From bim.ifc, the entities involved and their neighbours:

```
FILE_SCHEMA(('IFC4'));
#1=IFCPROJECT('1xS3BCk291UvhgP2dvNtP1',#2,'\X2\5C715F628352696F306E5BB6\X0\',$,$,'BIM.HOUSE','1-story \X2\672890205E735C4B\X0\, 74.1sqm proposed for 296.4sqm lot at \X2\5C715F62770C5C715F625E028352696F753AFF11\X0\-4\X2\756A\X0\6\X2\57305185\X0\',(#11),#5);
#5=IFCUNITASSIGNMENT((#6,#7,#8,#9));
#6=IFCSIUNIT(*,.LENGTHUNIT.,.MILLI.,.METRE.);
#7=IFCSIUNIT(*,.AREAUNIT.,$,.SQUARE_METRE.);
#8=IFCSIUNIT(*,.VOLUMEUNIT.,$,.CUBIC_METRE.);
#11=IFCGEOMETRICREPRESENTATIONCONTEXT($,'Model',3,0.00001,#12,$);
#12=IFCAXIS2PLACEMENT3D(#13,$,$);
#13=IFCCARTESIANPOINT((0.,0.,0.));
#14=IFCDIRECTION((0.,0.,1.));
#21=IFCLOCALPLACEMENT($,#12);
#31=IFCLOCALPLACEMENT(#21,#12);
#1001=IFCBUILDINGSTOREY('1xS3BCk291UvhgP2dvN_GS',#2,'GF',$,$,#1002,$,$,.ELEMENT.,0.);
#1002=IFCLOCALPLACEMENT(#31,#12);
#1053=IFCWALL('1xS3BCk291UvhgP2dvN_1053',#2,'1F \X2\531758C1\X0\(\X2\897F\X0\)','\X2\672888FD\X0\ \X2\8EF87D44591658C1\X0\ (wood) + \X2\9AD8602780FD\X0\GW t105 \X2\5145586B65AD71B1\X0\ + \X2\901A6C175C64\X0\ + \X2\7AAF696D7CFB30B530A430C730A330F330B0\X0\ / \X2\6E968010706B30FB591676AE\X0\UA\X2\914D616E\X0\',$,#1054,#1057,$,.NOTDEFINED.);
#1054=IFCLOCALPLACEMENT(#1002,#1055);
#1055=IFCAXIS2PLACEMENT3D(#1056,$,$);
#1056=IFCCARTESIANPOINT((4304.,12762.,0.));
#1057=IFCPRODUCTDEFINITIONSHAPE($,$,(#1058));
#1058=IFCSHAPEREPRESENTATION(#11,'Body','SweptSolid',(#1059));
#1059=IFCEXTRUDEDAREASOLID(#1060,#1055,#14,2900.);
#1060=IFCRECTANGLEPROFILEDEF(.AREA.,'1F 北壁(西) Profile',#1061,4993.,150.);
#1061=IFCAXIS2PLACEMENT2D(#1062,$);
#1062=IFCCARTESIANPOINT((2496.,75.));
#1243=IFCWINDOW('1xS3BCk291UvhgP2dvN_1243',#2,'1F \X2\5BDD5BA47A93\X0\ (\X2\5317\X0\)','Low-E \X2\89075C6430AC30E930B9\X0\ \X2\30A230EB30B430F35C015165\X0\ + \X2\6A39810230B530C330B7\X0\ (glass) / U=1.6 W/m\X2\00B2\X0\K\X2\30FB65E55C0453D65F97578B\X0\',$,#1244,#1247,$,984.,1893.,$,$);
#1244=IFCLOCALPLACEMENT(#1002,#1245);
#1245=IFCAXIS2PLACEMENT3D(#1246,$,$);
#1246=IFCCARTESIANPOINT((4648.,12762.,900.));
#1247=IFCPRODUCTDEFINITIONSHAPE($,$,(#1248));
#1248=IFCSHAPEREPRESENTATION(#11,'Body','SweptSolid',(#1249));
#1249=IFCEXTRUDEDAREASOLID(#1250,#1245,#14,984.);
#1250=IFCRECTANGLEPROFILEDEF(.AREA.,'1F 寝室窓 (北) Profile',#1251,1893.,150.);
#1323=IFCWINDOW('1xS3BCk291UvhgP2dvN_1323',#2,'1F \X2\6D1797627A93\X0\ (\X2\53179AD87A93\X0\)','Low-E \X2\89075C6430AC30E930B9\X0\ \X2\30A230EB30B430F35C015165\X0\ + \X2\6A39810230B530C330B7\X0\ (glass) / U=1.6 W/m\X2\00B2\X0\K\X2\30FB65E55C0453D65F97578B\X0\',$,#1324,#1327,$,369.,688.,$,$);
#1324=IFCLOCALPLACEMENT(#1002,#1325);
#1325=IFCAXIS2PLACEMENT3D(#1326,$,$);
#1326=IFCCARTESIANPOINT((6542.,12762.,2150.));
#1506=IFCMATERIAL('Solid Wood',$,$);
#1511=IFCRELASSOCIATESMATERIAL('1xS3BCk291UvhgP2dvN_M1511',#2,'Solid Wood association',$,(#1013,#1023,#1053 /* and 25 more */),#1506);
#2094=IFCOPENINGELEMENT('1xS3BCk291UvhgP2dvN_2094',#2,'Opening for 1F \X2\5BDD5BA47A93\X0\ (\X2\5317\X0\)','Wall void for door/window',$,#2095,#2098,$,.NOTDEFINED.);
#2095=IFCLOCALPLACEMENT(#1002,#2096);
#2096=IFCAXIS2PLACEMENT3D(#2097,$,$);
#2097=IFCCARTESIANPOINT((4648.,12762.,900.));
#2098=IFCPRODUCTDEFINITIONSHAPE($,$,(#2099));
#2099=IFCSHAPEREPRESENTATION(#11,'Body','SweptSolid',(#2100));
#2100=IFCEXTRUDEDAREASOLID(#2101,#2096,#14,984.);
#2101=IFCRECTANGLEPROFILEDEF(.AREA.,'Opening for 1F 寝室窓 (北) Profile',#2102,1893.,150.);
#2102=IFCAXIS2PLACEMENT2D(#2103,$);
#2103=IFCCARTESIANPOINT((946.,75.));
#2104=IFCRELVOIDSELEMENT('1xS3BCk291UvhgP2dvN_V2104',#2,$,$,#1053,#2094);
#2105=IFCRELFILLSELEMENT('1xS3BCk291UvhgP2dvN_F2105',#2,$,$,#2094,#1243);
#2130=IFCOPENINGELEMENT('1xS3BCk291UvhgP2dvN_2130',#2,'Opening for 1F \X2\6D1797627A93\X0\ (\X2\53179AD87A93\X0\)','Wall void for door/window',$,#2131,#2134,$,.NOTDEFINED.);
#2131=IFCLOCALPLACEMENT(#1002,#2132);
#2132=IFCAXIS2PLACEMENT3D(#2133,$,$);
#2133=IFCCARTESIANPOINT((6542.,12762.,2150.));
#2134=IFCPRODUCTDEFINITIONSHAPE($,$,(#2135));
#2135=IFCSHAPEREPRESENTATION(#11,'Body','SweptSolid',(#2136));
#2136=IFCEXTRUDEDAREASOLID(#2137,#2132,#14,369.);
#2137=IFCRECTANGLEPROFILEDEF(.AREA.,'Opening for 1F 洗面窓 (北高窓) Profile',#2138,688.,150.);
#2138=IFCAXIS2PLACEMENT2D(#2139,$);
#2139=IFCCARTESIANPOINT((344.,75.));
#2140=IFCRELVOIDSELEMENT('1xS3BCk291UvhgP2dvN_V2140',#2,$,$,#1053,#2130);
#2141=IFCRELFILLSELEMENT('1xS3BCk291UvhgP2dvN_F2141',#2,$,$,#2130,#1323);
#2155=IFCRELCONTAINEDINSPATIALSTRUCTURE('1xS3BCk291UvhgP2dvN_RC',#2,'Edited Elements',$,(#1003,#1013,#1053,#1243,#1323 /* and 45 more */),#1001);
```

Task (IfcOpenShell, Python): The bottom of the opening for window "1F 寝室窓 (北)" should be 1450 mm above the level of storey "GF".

```python
import numpy as np
import ifcopenshell
import ifcopenshell.api.geometry
import ifcopenshell.geom
import ifcopenshell.util.element
import ifcopenshell.util.placement
import ifcopenshell.util.shape
import ifcopenshell.util.unit

model = ifcopenshell.open("bim.ifc")
unit_scale = ifcopenshell.util.unit.calculate_unit_scale(model)

window = model.by_guid("1xS3BCk291UvhgP2dvN_1243")
opening = window.FillsVoids[0].RelatingOpeningElement
storey = ifcopenshell.util.element.get_container(window, ifc_class="IfcBuildingStorey")
level = ifcopenshell.util.placement.get_local_placement(storey.ObjectPlacement)[2, 3]

# The opening's origin need not be at the sill, so measure its lowest point.
shape = ifcopenshell.geom.create_shape(ifcopenshell.geom.settings(), opening)
bottom = ifcopenshell.util.shape.get_shape_bottom_elevation(shape, shape.geometry) / unit_scale
dz = level + 1.45 / unit_scale - bottom

shift = np.array([0.0, 0.0, dz])
# The window is not placed relative to its opening, so move both.
for product in (opening, window):
    matrix = ifcopenshell.util.placement.get_local_placement(product.ObjectPlacement)
    matrix[:3, 3] += shift
    ifcopenshell.api.geometry.edit_object_placement(model, product=product, matrix=matrix, is_si=False)

print(f"moved by {dz * unit_scale:+.3f} m")

model.write("bim-out.ifc")
```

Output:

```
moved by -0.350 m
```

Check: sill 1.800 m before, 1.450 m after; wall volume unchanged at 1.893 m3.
